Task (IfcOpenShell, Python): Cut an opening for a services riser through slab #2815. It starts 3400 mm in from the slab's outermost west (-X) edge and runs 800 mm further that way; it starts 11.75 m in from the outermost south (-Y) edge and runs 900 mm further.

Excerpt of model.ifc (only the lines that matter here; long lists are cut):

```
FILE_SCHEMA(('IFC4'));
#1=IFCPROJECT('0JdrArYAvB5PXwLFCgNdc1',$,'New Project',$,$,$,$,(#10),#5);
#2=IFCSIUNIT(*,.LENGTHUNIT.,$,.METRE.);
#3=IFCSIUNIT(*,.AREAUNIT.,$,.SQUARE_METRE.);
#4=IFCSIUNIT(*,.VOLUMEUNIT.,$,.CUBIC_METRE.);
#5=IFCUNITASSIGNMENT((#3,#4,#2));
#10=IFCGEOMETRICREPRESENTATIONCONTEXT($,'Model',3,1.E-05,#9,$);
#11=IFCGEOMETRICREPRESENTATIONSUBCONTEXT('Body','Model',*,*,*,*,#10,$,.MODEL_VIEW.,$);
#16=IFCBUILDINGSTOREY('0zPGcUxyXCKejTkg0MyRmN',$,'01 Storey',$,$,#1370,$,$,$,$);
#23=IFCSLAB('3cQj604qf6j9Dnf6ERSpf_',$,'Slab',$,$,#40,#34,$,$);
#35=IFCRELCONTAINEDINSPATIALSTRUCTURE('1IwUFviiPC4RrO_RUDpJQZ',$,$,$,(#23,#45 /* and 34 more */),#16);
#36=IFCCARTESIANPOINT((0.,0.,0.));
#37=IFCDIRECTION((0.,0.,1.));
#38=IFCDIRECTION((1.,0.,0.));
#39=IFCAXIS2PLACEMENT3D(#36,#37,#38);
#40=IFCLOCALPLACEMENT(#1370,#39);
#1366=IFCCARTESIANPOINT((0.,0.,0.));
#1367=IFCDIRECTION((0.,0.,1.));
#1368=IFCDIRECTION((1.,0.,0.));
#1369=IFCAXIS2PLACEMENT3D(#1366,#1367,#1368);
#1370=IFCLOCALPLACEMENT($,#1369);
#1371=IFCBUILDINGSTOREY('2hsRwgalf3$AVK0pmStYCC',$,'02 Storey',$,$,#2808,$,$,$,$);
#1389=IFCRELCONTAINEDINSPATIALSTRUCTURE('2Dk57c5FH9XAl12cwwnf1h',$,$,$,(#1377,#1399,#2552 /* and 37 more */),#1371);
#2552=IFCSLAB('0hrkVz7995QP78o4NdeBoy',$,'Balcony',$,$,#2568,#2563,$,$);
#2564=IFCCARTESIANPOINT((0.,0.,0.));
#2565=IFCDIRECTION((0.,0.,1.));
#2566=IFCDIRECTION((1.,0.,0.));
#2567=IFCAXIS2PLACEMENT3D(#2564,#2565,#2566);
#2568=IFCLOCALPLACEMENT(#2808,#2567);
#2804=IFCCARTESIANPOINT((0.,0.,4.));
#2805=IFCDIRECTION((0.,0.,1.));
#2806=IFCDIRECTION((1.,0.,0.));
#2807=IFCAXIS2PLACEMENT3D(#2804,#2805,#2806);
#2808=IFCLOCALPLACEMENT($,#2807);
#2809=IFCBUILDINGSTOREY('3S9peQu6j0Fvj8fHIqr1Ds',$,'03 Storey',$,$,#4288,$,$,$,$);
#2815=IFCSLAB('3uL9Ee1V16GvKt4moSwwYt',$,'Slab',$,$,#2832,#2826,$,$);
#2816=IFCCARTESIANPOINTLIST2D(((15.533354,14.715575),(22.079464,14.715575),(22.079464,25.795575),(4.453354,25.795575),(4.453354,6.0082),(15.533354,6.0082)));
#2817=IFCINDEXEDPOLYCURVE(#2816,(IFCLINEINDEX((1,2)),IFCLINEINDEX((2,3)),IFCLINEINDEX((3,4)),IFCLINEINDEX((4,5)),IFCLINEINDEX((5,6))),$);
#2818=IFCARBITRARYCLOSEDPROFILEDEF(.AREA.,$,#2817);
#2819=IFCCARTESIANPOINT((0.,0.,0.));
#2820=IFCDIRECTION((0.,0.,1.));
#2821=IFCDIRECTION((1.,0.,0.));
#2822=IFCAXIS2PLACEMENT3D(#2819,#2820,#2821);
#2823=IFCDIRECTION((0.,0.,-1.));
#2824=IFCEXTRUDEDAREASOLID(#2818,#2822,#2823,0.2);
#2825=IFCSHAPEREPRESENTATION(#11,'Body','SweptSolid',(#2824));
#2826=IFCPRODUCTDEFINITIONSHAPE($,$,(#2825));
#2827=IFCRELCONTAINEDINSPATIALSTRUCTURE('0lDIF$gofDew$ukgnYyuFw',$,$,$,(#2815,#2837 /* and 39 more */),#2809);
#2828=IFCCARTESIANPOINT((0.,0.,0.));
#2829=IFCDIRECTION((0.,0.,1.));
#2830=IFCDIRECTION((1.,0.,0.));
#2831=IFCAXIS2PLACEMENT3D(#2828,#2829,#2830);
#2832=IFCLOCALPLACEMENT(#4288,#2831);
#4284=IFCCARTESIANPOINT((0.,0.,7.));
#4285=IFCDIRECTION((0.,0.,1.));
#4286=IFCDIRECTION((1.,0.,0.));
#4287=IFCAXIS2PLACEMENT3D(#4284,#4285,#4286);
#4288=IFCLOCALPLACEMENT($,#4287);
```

```python
import numpy as np
import ifcopenshell
import ifcopenshell.api.feature
import ifcopenshell.api.geometry
import ifcopenshell.api.root
import ifcopenshell.geom
import ifcopenshell.util.placement
import ifcopenshell.util.representation
import ifcopenshell.util.shape
import ifcopenshell.util.unit

model = ifcopenshell.open("model.ifc")
unit_scale = ifcopenshell.util.unit.calculate_unit_scale(model)
settings = ifcopenshell.geom.settings()


def volume(element):
    """Net volume in cubic metres, openings subtracted."""
    shape = ifcopenshell.geom.create_shape(settings, element)
    return ifcopenshell.util.shape.get_volume(shape.geometry)


slab = model.by_guid("3uL9Ee1V16GvKt4moSwwYt")
before = volume(slab)

# Extent in the slab's own axes, in metres. The edges named are its -X and -Y sides.
slab_shape = ifcopenshell.geom.create_shape(settings, slab)
vertices = ifcopenshell.util.shape.get_vertices(slab_shape.geometry)
x_min, y_min, bottom = vertices.min(axis=0)
top = vertices[:, 2].max()

opening = ifcopenshell.api.root.create_entity(model, ifc_class="IfcOpeningElement", name="Services riser opening", predefined_type="OPENING")
context = ifcopenshell.util.representation.get_context(model, "Model", "Body", "MODEL_VIEW")
width, depth = 0.8, 0.9
outline = [(0.0, 0.0), (width, 0.0), (width, depth), (0.0, depth), (0.0, 0.0)]
# Overshoot both faces by 50 mm so the cut is clean.
shape = ifcopenshell.api.geometry.add_slab_representation(
    model, context=context, depth=top - bottom + 0.1, polyline=outline
)
ifcopenshell.api.geometry.assign_representation(model, product=opening, representation=shape)

matrix = ifcopenshell.util.placement.get_local_placement(slab.ObjectPlacement)
matrix[:, 3] = matrix @ np.append(np.array([x_min + 3.4, y_min + 11.75, bottom - 0.05]) / unit_scale, 1.0)
ifcopenshell.api.geometry.edit_object_placement(model, product=opening, matrix=matrix, is_si=False)
ifcopenshell.api.feature.add_feature(model, feature=opening, element=slab)

after = volume(slab)

print(f"slab volume {before:.3f} -> {after:.3f} m3")

model.write("model_updated.ifc")
```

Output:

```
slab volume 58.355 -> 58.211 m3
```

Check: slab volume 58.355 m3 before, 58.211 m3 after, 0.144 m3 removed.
